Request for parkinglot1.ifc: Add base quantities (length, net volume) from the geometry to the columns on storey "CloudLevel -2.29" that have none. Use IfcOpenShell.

First a look at what the model holds.

```python
import ifcopenshell
import ifcopenshell.util.element
import ifcopenshell.util.unit

model = ifcopenshell.open("parkinglot1.ifc")
print(model.schema)
for unit_type in ("LENGTHUNIT", "AREAUNIT", "VOLUMEUNIT"):
    print(unit_type, ifcopenshell.util.unit.calculate_unit_scale(model, unit_type))
storey = next(s for s in model.by_type("IfcBuildingStorey") if s.Name == "CloudLevel -2.29")
columns = [e for e in ifcopenshell.util.element.get_decomposition(storey) if e.is_a("IfcColumn")]
for e in sorted(columns, key=lambda e: e.id()):
    print(e.id(), e.is_a(), e.Name, list(ifcopenshell.util.element.get_psets(e, qtos_only=True)), sep=" | ")
```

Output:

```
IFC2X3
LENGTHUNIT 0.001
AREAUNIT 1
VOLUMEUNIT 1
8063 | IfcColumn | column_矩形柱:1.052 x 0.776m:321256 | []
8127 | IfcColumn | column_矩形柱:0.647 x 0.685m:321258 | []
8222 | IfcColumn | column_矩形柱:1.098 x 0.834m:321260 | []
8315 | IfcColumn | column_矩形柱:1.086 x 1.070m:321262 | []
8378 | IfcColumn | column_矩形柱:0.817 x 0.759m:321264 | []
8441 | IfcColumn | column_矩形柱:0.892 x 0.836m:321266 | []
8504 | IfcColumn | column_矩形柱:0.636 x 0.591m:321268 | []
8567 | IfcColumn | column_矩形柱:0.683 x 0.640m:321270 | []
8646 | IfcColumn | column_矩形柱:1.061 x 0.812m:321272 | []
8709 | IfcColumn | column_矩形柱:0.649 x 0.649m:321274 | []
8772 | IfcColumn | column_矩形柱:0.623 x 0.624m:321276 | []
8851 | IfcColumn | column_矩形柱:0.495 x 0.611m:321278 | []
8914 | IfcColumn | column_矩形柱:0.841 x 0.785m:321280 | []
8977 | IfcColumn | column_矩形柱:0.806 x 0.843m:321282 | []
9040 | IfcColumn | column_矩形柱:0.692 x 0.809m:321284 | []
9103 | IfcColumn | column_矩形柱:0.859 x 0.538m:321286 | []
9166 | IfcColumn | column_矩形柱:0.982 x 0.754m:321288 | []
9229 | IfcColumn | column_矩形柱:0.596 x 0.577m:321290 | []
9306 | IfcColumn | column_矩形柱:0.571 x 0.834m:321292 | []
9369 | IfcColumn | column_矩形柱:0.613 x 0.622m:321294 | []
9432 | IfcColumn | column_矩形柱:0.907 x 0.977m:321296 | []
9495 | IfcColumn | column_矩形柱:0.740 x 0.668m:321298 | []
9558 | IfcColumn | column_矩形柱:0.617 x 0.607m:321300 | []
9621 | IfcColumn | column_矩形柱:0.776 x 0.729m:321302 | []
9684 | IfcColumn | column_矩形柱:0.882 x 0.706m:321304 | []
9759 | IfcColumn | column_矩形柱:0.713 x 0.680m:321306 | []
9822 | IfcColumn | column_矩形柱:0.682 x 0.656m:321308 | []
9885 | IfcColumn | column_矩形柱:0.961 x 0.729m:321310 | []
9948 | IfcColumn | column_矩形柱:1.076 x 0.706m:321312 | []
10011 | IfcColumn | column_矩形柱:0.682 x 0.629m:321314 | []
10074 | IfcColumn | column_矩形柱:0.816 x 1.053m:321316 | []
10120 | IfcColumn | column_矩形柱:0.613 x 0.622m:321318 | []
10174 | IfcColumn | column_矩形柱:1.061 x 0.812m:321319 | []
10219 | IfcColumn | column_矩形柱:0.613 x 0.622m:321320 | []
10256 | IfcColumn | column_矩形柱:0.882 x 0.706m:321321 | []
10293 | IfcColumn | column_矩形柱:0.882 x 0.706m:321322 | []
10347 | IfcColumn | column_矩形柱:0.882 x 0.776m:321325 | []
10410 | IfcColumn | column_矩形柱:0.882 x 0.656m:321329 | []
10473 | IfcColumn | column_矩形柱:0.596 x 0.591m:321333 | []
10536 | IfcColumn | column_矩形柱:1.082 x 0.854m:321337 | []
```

```python
import ifcopenshell
import ifcopenshell.api.pset
import ifcopenshell.geom
import ifcopenshell.util.element
import ifcopenshell.util.shape
import ifcopenshell.util.unit

model = ifcopenshell.open("parkinglot1.ifc")
unit_scale = ifcopenshell.util.unit.calculate_unit_scale(model)
volume_scale = ifcopenshell.util.unit.calculate_unit_scale(model, "VOLUMEUNIT")
settings = ifcopenshell.geom.settings()

storey = next(s for s in model.by_type("IfcBuildingStorey") if s.Name == "CloudLevel -2.29")
columns = [e for e in ifcopenshell.util.element.get_decomposition(storey) if e.is_a("IfcColumn")]

for e in sorted(columns, key=lambda e: e.id()):
    if ifcopenshell.util.element.get_psets(e, qtos_only=True, should_inherit=False):
        continue
    # Geometry comes back in metres, in the element's own axes.
    shape = ifcopenshell.geom.create_shape(settings, e)
    values = {
        "Length": ifcopenshell.util.shape.get_z(shape.geometry) / unit_scale,
        "NetVolume": ifcopenshell.util.shape.get_volume(shape.geometry) / volume_scale,
    }
    qto = ifcopenshell.api.pset.add_qto(model, product=e, name="BaseQuantities")
    ifcopenshell.api.pset.edit_qto(model, qto=qto, properties=values)
    print(e.id(), {k: round(v, 3) for k, v in values.items()})

model.write("parkinglot1_updated.ifc")
```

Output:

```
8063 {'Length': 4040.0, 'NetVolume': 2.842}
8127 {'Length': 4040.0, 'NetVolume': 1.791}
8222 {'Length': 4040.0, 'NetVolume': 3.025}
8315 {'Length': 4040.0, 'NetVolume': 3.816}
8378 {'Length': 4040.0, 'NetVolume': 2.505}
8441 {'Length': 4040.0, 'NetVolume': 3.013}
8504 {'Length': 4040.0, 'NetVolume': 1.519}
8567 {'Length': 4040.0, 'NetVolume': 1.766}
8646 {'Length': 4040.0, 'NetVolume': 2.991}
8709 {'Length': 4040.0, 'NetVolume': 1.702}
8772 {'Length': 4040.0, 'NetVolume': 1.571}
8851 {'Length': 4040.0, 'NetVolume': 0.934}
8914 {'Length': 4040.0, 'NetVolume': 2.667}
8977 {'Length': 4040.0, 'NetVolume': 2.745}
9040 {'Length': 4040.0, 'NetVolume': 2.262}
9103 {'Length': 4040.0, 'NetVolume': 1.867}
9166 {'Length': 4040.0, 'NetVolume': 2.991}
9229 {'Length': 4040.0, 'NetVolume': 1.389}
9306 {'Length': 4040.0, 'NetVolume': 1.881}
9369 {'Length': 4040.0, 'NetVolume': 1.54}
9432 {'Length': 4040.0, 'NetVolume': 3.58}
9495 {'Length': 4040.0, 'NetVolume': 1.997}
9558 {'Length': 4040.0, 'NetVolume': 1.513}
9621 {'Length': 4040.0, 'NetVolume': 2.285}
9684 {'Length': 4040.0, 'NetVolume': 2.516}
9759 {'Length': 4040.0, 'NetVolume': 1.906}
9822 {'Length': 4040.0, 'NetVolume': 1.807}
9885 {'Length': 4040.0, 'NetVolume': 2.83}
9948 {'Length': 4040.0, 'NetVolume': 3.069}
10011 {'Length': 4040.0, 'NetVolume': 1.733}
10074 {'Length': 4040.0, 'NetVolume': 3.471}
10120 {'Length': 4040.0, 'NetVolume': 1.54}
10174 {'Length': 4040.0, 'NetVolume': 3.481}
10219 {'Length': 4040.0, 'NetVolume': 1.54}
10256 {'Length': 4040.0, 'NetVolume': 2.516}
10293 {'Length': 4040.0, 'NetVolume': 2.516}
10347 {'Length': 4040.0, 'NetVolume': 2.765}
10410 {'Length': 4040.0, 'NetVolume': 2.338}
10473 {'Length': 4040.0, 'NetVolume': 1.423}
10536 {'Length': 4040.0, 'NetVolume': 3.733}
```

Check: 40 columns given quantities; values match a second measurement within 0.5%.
